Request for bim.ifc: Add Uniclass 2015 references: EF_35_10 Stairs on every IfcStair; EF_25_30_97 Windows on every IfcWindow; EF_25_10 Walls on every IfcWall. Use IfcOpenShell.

First a look at what the model holds.

```python
import ifcopenshell

model = ifcopenshell.open("bim.ifc")
print(model.schema)
print("classifications:", [c.Name for c in model.by_type("IfcClassification")])
for ifc_class in ("IfcDoor", "IfcRoof", "IfcStair", "IfcWall", "IfcWindow"):
    print(ifc_class, len(model.by_type(ifc_class)))
```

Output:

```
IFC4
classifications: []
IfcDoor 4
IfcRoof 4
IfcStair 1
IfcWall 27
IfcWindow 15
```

```python
import ifcopenshell
import ifcopenshell.api.classification

model = ifcopenshell.open("bim.ifc")

system = ifcopenshell.api.classification.add_classification(model, classification="Uniclass 2015")

codes = {
    "IfcStair": ("EF_35_10", "Stairs"),
    "IfcWindow": ("EF_25_30_97", "Windows"),
    "IfcWall": ("EF_25_10", "Walls"),
}
for ifc_class, (code, name) in codes.items():
    products = model.by_type(ifc_class)
    ifcopenshell.api.classification.add_reference(
        model, products=products, classification=system, identification=code, name=name
    )
    print(code, len(products))

model.write("bim_v2.ifc")
```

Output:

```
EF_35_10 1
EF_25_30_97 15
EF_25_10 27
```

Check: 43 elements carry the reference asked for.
